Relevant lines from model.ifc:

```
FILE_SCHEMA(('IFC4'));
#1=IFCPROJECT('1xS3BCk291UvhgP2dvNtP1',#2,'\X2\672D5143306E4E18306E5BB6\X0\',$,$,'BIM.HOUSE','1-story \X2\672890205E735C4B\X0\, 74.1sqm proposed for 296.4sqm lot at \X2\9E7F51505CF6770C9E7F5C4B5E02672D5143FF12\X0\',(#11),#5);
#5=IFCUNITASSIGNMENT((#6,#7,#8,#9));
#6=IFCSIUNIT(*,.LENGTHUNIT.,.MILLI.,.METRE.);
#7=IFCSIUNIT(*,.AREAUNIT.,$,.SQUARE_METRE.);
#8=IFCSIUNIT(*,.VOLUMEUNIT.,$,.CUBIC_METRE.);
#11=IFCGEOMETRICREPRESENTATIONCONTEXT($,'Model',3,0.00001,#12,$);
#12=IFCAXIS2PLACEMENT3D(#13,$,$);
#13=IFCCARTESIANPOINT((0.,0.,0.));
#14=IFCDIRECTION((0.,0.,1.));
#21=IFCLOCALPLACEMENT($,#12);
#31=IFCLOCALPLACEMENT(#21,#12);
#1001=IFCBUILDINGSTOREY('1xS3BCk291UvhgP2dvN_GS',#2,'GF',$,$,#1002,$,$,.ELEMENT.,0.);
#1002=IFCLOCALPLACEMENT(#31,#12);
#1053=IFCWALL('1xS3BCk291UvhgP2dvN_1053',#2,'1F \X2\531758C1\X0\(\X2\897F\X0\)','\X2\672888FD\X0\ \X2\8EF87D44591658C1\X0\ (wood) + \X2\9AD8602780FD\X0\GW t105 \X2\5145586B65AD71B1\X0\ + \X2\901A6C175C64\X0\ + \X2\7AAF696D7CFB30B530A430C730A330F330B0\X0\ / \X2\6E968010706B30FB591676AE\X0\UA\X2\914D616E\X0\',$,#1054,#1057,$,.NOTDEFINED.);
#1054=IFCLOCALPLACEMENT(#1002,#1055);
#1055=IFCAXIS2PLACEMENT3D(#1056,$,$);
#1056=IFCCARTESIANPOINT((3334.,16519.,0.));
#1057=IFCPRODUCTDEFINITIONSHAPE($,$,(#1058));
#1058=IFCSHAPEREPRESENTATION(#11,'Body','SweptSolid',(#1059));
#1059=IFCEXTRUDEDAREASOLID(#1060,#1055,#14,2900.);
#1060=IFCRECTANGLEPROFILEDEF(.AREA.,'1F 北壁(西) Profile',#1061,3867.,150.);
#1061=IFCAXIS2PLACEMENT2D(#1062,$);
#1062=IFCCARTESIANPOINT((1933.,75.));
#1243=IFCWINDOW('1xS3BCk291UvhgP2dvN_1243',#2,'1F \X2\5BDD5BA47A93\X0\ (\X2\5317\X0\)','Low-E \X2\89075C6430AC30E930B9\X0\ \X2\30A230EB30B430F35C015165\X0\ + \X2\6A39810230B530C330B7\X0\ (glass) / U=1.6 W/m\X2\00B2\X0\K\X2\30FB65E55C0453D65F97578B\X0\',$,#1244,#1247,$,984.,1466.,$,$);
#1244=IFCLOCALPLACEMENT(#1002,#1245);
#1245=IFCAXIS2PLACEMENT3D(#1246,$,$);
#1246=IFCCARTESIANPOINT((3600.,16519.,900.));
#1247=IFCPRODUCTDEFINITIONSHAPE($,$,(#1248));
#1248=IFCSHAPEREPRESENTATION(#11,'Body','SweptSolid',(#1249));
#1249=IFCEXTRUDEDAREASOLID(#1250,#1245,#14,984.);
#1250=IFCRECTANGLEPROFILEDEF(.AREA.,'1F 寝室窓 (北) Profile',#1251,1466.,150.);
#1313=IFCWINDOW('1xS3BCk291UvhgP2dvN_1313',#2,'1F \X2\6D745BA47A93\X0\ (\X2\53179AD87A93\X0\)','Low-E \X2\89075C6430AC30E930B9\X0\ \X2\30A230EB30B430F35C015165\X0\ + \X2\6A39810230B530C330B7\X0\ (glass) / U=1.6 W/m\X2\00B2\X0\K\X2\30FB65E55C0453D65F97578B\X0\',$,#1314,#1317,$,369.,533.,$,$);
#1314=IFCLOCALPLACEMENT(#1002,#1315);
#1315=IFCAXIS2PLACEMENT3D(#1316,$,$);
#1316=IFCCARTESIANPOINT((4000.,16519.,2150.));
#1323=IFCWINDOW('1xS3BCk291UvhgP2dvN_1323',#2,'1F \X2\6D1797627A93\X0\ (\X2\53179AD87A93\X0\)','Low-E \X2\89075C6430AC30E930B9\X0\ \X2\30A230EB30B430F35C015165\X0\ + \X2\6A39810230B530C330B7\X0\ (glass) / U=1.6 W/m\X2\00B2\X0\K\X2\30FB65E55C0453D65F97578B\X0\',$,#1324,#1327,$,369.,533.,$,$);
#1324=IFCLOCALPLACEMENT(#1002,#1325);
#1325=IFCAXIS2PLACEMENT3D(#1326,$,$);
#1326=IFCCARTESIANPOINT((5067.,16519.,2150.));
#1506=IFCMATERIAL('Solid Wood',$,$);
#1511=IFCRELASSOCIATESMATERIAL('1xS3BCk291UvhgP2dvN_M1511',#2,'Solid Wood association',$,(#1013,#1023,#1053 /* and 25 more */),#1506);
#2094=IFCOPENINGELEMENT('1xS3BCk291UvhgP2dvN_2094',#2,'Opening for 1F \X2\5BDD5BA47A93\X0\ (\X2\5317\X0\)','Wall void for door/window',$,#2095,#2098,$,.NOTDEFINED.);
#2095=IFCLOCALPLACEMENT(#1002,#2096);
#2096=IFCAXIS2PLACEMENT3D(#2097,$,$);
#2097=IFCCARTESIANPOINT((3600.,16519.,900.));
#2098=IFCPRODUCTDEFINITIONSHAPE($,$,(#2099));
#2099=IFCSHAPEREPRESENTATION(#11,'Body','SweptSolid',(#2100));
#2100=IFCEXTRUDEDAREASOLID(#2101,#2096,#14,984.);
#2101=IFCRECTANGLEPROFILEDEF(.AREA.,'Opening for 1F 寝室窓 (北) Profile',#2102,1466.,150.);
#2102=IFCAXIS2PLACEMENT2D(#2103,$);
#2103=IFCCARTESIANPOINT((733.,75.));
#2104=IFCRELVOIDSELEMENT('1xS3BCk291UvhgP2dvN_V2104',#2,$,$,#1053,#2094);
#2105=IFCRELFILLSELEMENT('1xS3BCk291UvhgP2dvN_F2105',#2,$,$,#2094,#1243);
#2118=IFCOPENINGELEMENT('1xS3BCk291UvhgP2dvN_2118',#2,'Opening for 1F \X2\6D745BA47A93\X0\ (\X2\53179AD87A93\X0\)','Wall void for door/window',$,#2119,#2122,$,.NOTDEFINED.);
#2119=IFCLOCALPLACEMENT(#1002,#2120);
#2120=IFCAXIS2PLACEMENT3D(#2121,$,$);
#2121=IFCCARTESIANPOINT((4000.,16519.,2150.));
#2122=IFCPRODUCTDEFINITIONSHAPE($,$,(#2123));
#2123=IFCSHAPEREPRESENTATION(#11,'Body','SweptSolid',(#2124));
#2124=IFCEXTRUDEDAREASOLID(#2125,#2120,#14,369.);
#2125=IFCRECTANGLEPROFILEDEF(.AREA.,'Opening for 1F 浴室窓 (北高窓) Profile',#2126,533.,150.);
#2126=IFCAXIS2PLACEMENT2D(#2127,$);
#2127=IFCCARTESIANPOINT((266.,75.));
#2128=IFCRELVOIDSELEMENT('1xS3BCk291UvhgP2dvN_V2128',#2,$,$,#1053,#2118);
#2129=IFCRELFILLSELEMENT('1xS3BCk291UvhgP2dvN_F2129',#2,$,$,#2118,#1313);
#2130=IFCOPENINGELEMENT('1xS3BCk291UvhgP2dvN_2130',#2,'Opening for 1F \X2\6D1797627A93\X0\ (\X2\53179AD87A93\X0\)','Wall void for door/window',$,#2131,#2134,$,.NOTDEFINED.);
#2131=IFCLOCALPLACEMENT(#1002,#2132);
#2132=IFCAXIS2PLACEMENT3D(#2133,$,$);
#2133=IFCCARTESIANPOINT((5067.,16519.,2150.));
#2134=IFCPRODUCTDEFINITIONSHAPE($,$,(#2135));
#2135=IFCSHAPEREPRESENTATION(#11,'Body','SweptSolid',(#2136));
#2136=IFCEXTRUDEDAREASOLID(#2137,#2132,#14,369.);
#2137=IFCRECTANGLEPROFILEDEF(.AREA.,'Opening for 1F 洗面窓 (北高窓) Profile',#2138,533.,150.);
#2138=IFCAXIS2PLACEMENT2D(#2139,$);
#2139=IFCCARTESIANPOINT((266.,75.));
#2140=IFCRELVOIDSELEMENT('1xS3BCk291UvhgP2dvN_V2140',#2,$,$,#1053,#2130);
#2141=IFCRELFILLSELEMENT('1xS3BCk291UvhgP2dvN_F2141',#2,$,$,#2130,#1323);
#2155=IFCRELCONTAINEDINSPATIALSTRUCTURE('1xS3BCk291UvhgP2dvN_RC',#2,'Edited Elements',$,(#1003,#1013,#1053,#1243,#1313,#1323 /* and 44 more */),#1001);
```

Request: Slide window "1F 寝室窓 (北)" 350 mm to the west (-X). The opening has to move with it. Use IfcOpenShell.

```python
import ifcopenshell
import ifcopenshell.api.geometry
import ifcopenshell.util.placement

model = ifcopenshell.open("model.ifc")

window = model.by_guid("1xS3BCk291UvhgP2dvN_1243")
opening = window.FillsVoids[0].RelatingOpeningElement
wall = opening.VoidsElements[0].RelatingBuildingElement

wall_matrix = ifcopenshell.util.placement.get_local_placement(wall.ObjectPlacement)
shift = wall_matrix[:3, 0] * -350.0
before = ifcopenshell.util.placement.get_local_placement(window.ObjectPlacement)[:3, 3].copy()

# The window is not placed relative to its opening, so move both.
for product in (opening, window):
    matrix = ifcopenshell.util.placement.get_local_placement(product.ObjectPlacement)
    matrix[:3, 3] += shift
    ifcopenshell.api.geometry.edit_object_placement(model, product=product, matrix=matrix, is_si=False)

after = ifcopenshell.util.placement.get_local_placement(window.ObjectPlacement)[:3, 3]
print("window moved by", (after - before).round(3) + 0.0)

model.write("model_v2.ifc")
```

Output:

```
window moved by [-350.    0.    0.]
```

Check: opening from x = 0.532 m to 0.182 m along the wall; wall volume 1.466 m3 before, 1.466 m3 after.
